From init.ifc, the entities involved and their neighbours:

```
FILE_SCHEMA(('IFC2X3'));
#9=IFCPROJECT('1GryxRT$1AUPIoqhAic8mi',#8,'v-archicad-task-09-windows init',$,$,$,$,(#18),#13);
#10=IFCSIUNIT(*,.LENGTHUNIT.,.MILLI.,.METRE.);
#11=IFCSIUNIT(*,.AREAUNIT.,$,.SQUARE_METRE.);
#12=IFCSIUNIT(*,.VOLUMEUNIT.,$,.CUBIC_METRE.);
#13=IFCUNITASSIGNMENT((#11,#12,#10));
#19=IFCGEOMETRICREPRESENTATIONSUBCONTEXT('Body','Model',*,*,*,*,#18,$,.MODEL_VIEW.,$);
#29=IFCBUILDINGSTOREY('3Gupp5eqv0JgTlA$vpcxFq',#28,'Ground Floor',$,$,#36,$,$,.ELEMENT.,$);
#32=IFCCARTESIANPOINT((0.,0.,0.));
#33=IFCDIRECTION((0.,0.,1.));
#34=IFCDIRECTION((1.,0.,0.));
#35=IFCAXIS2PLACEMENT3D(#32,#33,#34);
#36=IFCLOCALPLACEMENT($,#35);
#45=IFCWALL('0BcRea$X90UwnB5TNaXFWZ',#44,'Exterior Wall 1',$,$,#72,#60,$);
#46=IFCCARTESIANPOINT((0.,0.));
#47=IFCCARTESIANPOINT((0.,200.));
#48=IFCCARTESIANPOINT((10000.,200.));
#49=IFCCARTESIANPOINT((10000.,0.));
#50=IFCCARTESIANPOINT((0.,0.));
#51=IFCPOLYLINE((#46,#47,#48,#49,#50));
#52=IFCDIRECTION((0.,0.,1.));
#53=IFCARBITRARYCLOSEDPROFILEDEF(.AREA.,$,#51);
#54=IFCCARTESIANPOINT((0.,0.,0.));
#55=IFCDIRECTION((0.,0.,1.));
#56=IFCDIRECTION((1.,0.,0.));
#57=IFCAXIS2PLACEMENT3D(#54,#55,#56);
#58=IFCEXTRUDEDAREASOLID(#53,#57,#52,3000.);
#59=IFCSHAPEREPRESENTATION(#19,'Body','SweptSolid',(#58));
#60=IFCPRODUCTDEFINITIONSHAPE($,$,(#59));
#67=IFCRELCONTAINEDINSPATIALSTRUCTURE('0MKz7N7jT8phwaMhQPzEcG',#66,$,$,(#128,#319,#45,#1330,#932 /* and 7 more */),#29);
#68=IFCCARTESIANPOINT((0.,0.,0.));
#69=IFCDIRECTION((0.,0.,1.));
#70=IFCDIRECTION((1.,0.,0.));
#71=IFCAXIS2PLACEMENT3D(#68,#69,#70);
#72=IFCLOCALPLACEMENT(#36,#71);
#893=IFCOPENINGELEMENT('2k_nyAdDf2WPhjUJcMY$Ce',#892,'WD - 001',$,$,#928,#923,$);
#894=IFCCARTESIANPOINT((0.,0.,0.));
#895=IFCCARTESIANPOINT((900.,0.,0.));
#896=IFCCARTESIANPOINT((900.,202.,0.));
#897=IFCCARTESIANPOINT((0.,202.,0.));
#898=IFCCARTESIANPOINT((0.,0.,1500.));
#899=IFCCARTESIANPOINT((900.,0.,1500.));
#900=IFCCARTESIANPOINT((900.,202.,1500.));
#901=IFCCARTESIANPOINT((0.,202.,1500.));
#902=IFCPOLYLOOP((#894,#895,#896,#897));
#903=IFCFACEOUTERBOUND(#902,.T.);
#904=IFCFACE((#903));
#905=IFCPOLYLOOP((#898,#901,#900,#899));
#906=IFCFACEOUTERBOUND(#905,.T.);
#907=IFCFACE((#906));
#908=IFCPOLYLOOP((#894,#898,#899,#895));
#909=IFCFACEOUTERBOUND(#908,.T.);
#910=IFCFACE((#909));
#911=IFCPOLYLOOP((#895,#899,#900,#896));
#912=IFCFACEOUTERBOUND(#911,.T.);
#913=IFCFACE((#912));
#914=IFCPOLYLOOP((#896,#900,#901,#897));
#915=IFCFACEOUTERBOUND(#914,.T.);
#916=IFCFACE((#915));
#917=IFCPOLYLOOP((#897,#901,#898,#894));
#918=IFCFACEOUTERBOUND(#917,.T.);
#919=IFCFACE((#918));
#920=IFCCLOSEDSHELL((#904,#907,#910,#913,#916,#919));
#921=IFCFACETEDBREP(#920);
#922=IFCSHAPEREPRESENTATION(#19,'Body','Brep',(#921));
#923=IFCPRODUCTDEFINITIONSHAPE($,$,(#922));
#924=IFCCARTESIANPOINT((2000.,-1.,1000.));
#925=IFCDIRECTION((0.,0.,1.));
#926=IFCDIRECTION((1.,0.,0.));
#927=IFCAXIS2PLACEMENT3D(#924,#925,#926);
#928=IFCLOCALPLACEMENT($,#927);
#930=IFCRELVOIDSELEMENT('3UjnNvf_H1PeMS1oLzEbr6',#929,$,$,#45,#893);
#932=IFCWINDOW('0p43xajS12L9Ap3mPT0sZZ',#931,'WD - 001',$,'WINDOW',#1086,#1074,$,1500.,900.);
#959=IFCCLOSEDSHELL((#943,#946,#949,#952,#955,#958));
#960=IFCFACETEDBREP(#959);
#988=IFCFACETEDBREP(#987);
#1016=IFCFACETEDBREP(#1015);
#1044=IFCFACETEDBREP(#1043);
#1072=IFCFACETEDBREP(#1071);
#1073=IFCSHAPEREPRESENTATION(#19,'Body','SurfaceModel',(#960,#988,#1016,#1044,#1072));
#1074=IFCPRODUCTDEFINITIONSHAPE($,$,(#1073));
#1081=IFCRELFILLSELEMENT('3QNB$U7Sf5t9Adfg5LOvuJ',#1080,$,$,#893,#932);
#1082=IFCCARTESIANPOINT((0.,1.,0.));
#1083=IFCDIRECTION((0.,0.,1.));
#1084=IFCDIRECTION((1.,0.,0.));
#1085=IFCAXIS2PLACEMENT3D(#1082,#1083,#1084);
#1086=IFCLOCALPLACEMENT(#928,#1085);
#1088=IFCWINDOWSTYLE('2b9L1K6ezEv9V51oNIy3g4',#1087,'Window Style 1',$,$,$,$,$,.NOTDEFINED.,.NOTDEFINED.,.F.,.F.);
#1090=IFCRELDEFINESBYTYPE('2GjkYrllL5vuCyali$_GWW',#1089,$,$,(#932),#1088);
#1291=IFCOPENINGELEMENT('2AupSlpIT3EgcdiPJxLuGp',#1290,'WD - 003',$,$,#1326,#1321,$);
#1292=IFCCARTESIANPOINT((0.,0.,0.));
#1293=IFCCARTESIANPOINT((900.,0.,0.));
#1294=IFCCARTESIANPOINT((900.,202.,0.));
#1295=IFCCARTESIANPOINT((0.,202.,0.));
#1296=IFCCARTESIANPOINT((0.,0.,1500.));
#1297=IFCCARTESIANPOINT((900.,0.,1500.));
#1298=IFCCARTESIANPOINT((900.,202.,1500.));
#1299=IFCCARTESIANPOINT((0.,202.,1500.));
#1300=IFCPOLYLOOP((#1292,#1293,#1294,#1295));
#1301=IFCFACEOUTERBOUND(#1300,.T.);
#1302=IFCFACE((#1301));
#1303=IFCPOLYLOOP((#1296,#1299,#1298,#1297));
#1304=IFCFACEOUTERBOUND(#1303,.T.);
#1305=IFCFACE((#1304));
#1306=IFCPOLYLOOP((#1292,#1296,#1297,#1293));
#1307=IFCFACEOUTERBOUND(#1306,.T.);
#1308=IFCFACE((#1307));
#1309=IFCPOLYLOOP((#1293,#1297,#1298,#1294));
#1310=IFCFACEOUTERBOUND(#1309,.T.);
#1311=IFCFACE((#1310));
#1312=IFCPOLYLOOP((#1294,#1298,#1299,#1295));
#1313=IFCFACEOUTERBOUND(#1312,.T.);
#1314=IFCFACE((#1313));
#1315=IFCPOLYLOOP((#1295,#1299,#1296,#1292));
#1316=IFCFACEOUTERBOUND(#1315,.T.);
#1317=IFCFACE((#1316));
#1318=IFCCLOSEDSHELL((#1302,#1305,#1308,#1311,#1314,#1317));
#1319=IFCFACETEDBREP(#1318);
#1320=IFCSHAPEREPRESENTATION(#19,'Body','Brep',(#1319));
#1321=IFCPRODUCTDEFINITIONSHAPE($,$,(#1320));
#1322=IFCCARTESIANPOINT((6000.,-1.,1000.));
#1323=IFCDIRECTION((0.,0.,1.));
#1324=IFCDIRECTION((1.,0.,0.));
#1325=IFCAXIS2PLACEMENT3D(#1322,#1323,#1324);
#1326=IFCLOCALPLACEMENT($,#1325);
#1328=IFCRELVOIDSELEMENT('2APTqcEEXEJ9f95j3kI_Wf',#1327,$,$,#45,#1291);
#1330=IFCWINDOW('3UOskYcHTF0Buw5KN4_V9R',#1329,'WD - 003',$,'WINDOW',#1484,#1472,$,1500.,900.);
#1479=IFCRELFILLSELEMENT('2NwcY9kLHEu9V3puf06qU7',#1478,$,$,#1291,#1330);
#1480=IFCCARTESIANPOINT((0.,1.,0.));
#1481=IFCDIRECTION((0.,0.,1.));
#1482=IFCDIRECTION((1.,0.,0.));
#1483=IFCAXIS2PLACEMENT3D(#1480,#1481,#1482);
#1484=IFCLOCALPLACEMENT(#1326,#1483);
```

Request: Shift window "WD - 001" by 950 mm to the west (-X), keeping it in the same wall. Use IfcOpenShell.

```python
import ifcopenshell
import ifcopenshell.api.geometry
import ifcopenshell.util.placement
import ifcopenshell.util.unit

model = ifcopenshell.open("init.ifc")
unit_scale = ifcopenshell.util.unit.calculate_unit_scale(model)

window = model.by_id(932)
opening = window.FillsVoids[0].RelatingOpeningElement
wall = opening.VoidsElements[0].RelatingBuildingElement

wall_matrix = ifcopenshell.util.placement.get_local_placement(wall.ObjectPlacement)
shift = wall_matrix[:3, 0] * -0.95 / unit_scale
before = ifcopenshell.util.placement.get_local_placement(window.ObjectPlacement)[:3, 3].copy()

# The window is placed relative to its opening, so it follows when the opening moves.
matrix = ifcopenshell.util.placement.get_local_placement(opening.ObjectPlacement)
matrix[:3, 3] += shift
ifcopenshell.api.geometry.edit_object_placement(
    model, product=opening, matrix=matrix, is_si=False, should_transform_children=True
)

after = ifcopenshell.util.placement.get_local_placement(window.ObjectPlacement)[:3, 3]
print("window moved by", (after - before).round(3) + 0.0)

model.write("init_v2.ifc")
```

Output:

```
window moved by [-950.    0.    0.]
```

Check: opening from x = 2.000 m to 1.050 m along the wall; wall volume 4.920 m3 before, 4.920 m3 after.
